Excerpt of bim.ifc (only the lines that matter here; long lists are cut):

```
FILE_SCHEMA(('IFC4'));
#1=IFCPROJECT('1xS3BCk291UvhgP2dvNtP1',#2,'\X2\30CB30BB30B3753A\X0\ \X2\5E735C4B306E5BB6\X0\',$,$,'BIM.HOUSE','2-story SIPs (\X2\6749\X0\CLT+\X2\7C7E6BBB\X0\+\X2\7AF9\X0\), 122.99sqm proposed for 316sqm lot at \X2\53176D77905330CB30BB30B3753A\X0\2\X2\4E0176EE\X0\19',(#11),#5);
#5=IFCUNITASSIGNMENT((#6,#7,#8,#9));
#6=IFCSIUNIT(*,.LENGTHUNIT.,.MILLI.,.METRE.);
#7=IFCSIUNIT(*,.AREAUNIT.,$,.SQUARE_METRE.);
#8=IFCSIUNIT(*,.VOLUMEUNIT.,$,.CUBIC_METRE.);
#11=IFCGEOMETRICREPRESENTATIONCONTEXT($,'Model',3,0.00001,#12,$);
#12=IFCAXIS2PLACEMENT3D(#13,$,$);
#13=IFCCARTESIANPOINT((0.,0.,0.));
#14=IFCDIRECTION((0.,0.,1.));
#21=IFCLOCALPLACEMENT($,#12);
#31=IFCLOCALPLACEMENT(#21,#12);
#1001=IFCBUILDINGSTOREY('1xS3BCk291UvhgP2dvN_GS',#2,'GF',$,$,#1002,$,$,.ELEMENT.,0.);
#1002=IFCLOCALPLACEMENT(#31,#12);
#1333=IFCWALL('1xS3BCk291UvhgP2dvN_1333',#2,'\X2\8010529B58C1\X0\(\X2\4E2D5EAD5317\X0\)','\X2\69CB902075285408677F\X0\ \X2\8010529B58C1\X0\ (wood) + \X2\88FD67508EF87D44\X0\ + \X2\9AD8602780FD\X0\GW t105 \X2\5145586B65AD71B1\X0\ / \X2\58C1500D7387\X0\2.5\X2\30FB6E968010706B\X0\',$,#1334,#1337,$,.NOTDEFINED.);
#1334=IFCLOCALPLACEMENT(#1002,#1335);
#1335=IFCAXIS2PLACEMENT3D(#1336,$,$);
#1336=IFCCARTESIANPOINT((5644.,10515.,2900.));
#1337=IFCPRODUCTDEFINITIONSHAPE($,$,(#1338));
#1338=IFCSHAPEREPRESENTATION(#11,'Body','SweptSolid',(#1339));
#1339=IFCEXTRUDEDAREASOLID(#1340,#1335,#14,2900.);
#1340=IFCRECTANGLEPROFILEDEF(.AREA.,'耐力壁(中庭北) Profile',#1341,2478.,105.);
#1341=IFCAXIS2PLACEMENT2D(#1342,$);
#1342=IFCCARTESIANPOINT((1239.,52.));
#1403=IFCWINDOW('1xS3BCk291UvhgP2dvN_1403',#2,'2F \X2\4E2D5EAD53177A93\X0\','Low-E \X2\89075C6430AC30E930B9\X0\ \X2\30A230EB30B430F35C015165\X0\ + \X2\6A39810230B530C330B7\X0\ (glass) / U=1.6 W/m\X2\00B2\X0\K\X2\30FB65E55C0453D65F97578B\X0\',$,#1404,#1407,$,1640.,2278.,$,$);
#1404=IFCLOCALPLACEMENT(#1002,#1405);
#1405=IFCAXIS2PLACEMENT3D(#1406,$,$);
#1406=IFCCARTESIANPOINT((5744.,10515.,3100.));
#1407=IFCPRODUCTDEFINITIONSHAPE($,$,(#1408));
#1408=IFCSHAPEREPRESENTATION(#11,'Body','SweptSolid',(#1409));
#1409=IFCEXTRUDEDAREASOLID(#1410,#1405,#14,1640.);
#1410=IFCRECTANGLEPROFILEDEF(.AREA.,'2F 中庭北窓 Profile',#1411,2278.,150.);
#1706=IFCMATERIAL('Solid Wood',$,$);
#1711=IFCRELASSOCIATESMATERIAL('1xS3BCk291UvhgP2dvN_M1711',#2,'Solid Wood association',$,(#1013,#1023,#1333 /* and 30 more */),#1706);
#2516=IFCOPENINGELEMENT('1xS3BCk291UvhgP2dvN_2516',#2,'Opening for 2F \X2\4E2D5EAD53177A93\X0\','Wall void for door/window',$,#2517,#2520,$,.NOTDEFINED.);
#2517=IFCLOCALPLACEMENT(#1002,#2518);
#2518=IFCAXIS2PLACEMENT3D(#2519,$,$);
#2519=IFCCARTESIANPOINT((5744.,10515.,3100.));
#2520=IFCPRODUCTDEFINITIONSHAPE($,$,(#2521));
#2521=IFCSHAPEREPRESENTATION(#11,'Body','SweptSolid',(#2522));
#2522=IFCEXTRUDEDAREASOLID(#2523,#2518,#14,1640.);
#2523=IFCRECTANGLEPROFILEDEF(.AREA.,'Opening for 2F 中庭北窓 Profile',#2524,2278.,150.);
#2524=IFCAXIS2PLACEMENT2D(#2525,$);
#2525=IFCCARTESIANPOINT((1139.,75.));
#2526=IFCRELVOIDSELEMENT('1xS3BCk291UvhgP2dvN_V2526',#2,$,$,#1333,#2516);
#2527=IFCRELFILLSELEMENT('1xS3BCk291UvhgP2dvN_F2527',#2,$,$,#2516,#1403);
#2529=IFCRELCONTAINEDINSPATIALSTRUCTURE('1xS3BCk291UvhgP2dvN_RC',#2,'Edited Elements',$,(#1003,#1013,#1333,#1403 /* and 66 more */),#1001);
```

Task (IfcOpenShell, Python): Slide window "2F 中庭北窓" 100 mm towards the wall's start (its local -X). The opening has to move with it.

```python
import ifcopenshell
import ifcopenshell.api.geometry
import ifcopenshell.util.placement
import ifcopenshell.util.unit

model = ifcopenshell.open("bim.ifc")
unit_scale = ifcopenshell.util.unit.calculate_unit_scale(model)

window = model.by_guid("1xS3BCk291UvhgP2dvN_1403")
opening = window.FillsVoids[0].RelatingOpeningElement
wall = opening.VoidsElements[0].RelatingBuildingElement

wall_matrix = ifcopenshell.util.placement.get_local_placement(wall.ObjectPlacement)
shift = wall_matrix[:3, 0] * -0.1 / unit_scale
before = ifcopenshell.util.placement.get_local_placement(window.ObjectPlacement)[:3, 3].copy()

# The window is not placed relative to its opening, so move both.
for product in (opening, window):
    matrix = ifcopenshell.util.placement.get_local_placement(product.ObjectPlacement)
    matrix[:3, 3] += shift
    ifcopenshell.api.geometry.edit_object_placement(model, product=product, matrix=matrix, is_si=False)

after = ifcopenshell.util.placement.get_local_placement(window.ObjectPlacement)[:3, 3]
print("window moved by", (after - before).round(3) + 0.0)

model.write("bim-out.ifc")
```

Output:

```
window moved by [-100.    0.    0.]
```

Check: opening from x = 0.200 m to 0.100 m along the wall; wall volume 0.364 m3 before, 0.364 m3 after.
